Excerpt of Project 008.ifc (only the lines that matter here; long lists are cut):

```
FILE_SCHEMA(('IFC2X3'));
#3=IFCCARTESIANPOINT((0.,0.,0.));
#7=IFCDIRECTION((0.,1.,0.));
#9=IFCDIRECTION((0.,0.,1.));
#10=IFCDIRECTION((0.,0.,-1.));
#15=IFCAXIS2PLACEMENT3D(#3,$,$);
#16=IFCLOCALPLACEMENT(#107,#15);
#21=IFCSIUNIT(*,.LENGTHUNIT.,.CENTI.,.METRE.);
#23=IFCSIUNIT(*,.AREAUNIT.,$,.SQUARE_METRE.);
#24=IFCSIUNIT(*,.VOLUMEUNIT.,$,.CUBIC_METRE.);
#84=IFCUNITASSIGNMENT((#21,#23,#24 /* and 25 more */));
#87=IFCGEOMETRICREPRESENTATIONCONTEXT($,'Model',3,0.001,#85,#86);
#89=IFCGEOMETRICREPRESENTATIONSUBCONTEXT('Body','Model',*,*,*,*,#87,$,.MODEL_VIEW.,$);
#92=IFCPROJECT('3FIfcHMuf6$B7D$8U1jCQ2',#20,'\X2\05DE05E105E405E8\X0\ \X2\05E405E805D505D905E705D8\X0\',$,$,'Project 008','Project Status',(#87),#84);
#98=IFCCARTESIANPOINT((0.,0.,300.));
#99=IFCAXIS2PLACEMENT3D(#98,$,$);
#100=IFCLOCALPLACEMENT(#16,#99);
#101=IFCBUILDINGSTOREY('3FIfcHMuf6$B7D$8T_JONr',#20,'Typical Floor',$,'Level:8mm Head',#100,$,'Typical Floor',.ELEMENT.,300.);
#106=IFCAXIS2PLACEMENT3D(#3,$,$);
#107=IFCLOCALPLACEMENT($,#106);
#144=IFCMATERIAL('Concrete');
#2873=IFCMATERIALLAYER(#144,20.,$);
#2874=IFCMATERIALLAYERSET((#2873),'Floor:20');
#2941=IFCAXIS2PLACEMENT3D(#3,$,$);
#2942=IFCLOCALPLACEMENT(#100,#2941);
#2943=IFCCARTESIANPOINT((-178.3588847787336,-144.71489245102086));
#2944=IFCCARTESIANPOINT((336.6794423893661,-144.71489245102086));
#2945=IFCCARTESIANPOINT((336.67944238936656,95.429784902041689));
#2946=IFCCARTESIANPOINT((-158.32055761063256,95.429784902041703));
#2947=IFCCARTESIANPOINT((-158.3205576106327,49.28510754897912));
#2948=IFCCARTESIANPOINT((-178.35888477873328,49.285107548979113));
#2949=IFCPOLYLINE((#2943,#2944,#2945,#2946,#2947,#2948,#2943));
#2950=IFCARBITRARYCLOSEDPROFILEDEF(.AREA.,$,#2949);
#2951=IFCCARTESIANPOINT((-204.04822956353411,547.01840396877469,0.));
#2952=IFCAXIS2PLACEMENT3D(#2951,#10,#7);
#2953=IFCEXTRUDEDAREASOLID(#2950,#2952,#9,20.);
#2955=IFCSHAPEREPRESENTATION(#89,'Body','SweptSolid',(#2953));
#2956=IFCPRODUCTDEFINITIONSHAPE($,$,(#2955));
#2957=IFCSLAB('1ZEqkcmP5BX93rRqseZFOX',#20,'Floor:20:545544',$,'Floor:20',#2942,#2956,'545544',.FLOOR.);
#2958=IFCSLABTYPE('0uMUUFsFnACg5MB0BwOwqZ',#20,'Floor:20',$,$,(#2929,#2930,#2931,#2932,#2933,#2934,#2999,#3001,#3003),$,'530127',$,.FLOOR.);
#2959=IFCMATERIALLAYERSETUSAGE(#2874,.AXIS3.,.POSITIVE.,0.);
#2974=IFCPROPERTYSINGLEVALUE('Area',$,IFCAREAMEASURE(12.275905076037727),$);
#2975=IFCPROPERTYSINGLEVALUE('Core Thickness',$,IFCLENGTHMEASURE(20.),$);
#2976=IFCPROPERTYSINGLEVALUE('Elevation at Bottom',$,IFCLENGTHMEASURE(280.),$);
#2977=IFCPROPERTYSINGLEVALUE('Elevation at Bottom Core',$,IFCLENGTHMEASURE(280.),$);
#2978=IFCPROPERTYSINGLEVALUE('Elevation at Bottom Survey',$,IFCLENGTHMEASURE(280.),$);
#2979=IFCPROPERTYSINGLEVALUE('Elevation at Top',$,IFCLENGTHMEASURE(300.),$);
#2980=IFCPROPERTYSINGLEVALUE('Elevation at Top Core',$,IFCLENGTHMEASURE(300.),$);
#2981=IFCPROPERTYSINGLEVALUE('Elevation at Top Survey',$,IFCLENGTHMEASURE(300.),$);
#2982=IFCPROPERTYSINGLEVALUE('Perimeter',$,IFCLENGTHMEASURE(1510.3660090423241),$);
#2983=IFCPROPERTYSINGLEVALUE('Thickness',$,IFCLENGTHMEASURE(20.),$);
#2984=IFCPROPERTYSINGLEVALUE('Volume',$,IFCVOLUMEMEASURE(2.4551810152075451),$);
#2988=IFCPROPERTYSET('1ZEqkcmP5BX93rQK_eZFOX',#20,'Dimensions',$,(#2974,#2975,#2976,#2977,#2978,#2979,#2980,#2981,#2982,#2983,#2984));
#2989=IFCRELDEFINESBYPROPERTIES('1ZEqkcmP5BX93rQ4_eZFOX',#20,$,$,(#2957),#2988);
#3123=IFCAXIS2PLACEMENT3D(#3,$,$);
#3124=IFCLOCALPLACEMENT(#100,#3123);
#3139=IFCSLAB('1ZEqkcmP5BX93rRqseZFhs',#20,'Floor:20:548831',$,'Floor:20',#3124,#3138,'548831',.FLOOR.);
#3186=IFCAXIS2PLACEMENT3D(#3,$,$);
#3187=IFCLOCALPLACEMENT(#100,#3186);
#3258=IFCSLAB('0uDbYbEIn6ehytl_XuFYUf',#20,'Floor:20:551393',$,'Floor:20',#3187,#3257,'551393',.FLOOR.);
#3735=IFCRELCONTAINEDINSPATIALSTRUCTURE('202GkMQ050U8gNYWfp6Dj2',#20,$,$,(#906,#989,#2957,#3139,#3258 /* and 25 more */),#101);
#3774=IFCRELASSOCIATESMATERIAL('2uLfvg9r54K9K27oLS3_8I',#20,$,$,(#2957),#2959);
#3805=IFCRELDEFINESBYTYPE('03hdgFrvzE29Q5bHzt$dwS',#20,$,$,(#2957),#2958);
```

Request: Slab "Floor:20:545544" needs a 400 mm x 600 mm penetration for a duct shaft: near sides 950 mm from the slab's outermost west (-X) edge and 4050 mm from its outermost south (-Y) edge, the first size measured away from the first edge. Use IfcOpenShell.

```python
import numpy as np
import ifcopenshell
import ifcopenshell.api.feature
import ifcopenshell.api.geometry
import ifcopenshell.api.pset
import ifcopenshell.api.root
import ifcopenshell.geom
import ifcopenshell.util.element
import ifcopenshell.util.placement
import ifcopenshell.util.representation
import ifcopenshell.util.shape
import ifcopenshell.util.unit

model = ifcopenshell.open("Project 008.ifc")
unit_scale = ifcopenshell.util.unit.calculate_unit_scale(model)
area_scale = ifcopenshell.util.unit.calculate_unit_scale(model, "AREAUNIT")
volume_scale = ifcopenshell.util.unit.calculate_unit_scale(model, "VOLUMEUNIT")
settings = ifcopenshell.geom.settings()


def volume(element):
    """Net volume in cubic metres, openings subtracted."""
    shape = ifcopenshell.geom.create_shape(settings, element)
    return ifcopenshell.util.shape.get_volume(shape.geometry)


slab = model.by_guid("1ZEqkcmP5BX93rRqseZFOX")
before = volume(slab)

# Extent in the slab's own axes, in metres. The edges named are its -X and -Y sides.
slab_shape = ifcopenshell.geom.create_shape(settings, slab)
vertices = ifcopenshell.util.shape.get_vertices(slab_shape.geometry)
x_min, y_min, bottom = vertices.min(axis=0)
top = vertices[:, 2].max()

opening = ifcopenshell.api.root.create_entity(model, ifc_class="IfcOpeningElement", name="Duct shaft opening")
context = ifcopenshell.util.representation.get_context(model, "Model", "Body", "MODEL_VIEW")
width, depth = 0.4, 0.6
outline = [(0.0, 0.0), (width, 0.0), (width, depth), (0.0, depth), (0.0, 0.0)]
# Overshoot both faces by 50 mm so the cut is clean.
shape = ifcopenshell.api.geometry.add_slab_representation(
    model, context=context, depth=top - bottom + 0.1, polyline=outline
)
ifcopenshell.api.geometry.assign_representation(model, product=opening, representation=shape)

matrix = ifcopenshell.util.placement.get_local_placement(slab.ObjectPlacement)
matrix[:, 3] = matrix @ np.append(np.array([x_min + 0.95, y_min + 4.05, bottom - 0.05]) / unit_scale, 1.0)
ifcopenshell.api.geometry.edit_object_placement(model, product=opening, matrix=matrix, is_si=False)
ifcopenshell.api.feature.add_feature(model, feature=opening, element=slab)

after = volume(slab)

# Update the slab's stored quantities.
pset = model.by_id(ifcopenshell.util.element.get_pset(slab, "Dimensions", should_inherit=False)["id"])
ifcopenshell.api.pset.edit_pset(model, pset=pset, properties={
    "Area": model.create_entity("IfcAreaMeasure", after / (top - bottom) / area_scale),
    "Volume": model.create_entity("IfcVolumeMeasure", after / volume_scale),
})

print(f"slab volume {before:.3f} -> {after:.3f} m3")

model.write("Project 008_updated.ifc")
```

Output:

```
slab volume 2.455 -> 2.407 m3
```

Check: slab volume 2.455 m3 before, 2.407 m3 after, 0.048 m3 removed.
